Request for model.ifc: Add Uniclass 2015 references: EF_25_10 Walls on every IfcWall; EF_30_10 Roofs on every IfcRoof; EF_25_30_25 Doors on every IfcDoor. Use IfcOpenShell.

First a look at what the model holds.

```python
import ifcopenshell

model = ifcopenshell.open("model.ifc")
print(model.schema)
print("classifications:", [c.Name for c in model.by_type("IfcClassification")])
for ifc_class in ("IfcDoor", "IfcRoof", "IfcStair", "IfcWall", "IfcWindow"):
    print(ifc_class, len(model.by_type(ifc_class)))
```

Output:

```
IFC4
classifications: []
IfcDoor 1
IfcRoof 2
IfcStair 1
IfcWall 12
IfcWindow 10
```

```python
import ifcopenshell
import ifcopenshell.api.classification

model = ifcopenshell.open("model.ifc")

system = ifcopenshell.api.classification.add_classification(model, classification="Uniclass 2015")

codes = {
    "IfcWall": ("EF_25_10", "Walls"),
    "IfcRoof": ("EF_30_10", "Roofs"),
    "IfcDoor": ("EF_25_30_25", "Doors"),
}
for ifc_class, (code, name) in codes.items():
    products = model.by_type(ifc_class)
    ifcopenshell.api.classification.add_reference(
        model, products=products, classification=system, identification=code, name=name
    )
    print(code, len(products))

model.write("model_rev.ifc")
```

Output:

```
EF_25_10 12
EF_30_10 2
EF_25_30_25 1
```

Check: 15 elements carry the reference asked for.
